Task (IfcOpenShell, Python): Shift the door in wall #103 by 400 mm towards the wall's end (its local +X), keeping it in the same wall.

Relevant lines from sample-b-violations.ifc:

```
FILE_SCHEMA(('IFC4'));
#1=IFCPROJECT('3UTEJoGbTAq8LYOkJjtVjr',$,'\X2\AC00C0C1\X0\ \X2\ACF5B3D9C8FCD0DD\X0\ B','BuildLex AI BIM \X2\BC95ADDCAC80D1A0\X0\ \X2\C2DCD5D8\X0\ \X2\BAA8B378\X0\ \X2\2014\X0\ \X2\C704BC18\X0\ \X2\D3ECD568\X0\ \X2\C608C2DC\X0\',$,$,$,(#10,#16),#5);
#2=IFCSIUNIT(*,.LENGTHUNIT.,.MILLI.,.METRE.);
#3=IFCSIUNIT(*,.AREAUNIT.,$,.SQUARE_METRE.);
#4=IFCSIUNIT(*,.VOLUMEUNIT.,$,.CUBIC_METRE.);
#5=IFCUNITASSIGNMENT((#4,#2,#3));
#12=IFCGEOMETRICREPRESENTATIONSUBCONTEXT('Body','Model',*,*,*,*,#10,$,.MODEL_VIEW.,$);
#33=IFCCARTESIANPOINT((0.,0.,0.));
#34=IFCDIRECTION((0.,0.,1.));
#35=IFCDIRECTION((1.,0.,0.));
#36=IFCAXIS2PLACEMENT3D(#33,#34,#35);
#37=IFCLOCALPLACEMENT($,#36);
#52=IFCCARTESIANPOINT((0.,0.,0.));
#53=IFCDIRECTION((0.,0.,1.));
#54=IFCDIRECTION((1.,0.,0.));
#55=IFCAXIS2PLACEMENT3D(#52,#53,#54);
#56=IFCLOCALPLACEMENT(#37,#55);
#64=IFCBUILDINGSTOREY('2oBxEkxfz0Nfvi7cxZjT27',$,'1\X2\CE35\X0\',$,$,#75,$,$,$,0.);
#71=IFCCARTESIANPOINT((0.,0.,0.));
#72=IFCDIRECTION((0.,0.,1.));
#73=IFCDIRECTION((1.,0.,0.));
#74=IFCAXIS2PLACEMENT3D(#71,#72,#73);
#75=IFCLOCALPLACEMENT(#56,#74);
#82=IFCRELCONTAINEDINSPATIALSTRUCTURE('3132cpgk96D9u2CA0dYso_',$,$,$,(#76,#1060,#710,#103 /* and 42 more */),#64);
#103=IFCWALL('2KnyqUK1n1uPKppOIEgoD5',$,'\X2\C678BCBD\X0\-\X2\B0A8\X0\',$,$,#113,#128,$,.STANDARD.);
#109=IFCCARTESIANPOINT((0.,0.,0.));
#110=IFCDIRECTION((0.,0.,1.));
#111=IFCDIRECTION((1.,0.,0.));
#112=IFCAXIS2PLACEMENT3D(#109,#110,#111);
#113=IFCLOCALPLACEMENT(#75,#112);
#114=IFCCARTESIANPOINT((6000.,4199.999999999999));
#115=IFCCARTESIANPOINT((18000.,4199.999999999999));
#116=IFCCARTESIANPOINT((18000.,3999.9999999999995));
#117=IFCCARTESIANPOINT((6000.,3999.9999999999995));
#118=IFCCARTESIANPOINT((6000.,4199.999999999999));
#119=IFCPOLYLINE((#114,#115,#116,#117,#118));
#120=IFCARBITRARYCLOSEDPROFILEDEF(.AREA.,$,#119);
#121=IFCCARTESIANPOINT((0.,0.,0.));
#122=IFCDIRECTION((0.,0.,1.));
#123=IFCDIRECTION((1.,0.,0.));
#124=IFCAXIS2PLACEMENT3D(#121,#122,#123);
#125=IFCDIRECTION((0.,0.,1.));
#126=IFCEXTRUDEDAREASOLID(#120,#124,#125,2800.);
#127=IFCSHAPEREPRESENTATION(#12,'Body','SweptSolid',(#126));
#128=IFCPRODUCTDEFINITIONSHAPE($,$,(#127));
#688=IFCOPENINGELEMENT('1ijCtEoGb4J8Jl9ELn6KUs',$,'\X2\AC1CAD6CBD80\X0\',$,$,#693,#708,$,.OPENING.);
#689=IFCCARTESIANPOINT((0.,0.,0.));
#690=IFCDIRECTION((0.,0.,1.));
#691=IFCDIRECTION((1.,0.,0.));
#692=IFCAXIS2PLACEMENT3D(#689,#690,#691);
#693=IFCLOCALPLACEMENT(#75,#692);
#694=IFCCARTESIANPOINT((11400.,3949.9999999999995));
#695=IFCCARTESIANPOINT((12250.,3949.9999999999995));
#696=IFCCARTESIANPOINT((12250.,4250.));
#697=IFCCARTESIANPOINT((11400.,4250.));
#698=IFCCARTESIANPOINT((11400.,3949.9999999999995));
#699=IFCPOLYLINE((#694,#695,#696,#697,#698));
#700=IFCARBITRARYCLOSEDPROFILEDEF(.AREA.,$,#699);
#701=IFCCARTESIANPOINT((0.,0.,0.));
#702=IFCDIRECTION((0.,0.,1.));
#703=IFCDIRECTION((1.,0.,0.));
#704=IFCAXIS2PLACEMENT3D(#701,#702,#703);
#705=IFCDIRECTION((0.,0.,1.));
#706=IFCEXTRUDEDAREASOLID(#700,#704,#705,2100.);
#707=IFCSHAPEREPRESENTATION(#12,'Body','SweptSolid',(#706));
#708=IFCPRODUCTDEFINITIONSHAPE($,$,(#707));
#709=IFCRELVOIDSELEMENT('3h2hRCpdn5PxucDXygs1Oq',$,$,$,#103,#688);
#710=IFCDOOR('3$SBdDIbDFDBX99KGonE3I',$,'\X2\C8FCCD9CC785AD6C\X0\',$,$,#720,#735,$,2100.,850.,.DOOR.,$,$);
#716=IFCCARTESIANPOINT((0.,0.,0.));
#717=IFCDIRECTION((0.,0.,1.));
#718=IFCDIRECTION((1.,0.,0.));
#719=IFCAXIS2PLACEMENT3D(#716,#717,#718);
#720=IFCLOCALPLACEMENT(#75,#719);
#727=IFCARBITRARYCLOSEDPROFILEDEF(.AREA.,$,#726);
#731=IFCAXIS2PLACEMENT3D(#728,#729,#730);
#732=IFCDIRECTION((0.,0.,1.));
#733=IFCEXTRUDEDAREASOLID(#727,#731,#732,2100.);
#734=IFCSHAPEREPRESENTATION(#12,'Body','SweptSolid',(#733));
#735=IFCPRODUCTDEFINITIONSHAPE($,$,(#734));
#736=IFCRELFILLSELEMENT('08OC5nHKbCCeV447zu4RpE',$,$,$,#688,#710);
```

```python
import ifcopenshell
import ifcopenshell.api.geometry
import ifcopenshell.util.placement

model = ifcopenshell.open("sample-b-violations.ifc")

door = model.by_id(710)
opening = door.FillsVoids[0].RelatingOpeningElement
wall = opening.VoidsElements[0].RelatingBuildingElement

wall_matrix = ifcopenshell.util.placement.get_local_placement(wall.ObjectPlacement)
shift = wall_matrix[:3, 0] * 400.0
before = ifcopenshell.util.placement.get_local_placement(door.ObjectPlacement)[:3, 3].copy()

# The door is not placed relative to its opening, so move both.
for product in (opening, door):
    matrix = ifcopenshell.util.placement.get_local_placement(product.ObjectPlacement)
    matrix[:3, 3] += shift
    ifcopenshell.api.geometry.edit_object_placement(model, product=product, matrix=matrix, is_si=False)

after = ifcopenshell.util.placement.get_local_placement(door.ObjectPlacement)[:3, 3]
print("door moved by", (after - before).round(3) + 0.0)

model.write("sample-b-violations-out.ifc")
```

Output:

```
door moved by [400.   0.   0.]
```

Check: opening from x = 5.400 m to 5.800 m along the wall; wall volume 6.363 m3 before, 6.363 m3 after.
